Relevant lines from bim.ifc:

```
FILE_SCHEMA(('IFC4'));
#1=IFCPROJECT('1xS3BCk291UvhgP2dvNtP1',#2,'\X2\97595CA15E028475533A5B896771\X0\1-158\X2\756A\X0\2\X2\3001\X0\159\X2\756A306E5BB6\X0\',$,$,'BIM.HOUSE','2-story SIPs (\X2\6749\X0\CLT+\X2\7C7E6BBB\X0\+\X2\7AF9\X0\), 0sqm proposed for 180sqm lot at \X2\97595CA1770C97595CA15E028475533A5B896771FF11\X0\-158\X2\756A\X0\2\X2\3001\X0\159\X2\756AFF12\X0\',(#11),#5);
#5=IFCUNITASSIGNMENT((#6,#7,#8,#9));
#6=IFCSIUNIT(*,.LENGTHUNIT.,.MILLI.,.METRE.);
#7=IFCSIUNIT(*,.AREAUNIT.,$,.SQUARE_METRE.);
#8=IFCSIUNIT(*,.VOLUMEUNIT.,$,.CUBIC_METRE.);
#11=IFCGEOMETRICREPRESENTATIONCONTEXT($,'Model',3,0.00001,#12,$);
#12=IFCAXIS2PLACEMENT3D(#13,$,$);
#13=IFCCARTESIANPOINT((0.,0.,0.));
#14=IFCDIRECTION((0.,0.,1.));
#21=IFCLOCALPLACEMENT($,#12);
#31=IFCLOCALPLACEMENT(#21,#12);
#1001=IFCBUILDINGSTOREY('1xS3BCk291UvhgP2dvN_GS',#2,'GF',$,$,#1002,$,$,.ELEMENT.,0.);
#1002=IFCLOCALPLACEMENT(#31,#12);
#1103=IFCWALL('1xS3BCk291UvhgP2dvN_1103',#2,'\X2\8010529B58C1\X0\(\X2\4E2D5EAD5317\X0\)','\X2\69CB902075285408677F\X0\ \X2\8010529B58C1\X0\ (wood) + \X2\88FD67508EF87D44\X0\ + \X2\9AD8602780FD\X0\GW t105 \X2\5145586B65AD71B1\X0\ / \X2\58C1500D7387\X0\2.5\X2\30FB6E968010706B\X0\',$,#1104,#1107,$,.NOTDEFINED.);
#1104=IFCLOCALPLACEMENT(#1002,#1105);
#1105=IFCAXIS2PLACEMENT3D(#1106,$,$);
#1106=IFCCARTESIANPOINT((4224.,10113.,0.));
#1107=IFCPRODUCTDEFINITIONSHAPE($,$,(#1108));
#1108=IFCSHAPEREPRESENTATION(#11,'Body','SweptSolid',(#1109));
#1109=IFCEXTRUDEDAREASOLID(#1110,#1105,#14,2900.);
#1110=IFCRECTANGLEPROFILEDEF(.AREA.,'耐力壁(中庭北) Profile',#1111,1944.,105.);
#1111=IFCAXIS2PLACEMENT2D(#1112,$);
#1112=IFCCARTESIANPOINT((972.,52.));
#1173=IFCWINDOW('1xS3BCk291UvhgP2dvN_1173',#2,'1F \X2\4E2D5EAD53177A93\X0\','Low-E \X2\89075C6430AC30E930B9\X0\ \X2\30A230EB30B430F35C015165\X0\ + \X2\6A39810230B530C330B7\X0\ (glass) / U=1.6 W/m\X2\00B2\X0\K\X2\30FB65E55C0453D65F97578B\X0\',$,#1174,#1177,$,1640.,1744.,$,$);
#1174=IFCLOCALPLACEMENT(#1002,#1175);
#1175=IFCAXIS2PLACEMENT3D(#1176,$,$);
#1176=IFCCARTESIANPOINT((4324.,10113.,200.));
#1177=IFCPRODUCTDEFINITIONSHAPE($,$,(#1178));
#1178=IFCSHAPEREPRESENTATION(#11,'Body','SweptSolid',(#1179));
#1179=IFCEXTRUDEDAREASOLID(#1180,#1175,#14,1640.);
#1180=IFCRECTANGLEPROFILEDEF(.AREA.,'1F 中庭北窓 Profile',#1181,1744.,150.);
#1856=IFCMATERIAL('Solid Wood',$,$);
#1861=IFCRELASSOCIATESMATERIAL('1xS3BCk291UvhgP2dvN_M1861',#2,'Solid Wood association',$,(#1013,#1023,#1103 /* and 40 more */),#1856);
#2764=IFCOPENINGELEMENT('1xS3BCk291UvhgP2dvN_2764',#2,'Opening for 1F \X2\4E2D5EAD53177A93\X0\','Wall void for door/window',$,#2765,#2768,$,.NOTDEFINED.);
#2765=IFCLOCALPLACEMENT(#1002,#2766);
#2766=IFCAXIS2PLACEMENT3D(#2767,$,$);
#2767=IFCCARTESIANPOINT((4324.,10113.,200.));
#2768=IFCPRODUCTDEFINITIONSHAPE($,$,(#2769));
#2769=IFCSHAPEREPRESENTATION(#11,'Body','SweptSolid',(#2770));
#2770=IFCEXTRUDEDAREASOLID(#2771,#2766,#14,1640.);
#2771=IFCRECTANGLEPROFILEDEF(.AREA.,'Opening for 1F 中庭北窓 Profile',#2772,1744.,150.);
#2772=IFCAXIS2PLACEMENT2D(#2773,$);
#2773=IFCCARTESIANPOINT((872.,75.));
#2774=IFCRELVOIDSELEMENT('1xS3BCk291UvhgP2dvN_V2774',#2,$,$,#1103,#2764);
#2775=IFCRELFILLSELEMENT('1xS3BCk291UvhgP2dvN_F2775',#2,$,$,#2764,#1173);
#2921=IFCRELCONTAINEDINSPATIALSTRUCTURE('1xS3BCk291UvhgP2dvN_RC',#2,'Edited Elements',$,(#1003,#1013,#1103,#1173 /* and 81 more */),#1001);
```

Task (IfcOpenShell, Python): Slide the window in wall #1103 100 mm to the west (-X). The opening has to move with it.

```python
import ifcopenshell
import ifcopenshell.api.geometry
import ifcopenshell.util.placement
import ifcopenshell.util.unit

model = ifcopenshell.open("bim.ifc")
unit_scale = ifcopenshell.util.unit.calculate_unit_scale(model)

window = model.by_guid("1xS3BCk291UvhgP2dvN_1173")
opening = window.FillsVoids[0].RelatingOpeningElement
wall = opening.VoidsElements[0].RelatingBuildingElement

wall_matrix = ifcopenshell.util.placement.get_local_placement(wall.ObjectPlacement)
shift = wall_matrix[:3, 0] * -0.1 / unit_scale
before = ifcopenshell.util.placement.get_local_placement(window.ObjectPlacement)[:3, 3].copy()

# The window is not placed relative to its opening, so move both.
for product in (opening, window):
    matrix = ifcopenshell.util.placement.get_local_placement(product.ObjectPlacement)
    matrix[:3, 3] += shift
    ifcopenshell.api.geometry.edit_object_placement(model, product=product, matrix=matrix, is_si=False)

after = ifcopenshell.util.placement.get_local_placement(window.ObjectPlacement)[:3, 3]
print("window moved by", (after - before).round(3) + 0.0)

model.write("bim_updated.ifc")
```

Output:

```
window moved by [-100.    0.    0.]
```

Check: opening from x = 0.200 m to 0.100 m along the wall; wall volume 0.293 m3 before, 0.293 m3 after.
